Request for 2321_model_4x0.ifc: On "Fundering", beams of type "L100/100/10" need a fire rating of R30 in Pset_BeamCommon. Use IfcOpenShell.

First a look at what the model holds.

```python
import ifcopenshell
import ifcopenshell.util.element

model = ifcopenshell.open("2321_model_4x0.ifc")
print(model.schema)
storey = next(s for s in model.by_type("IfcBuildingStorey") if s.Name == "Fundering")
beams = [e for e in ifcopenshell.util.element.get_decomposition(storey) if e.is_a("IfcBeam")]
seen = {}
for e in beams:
    element_type = ifcopenshell.util.element.get_type(e)
    key = (element_type.Name if element_type != e and element_type else None, ifcopenshell.util.element.get_pset(e, "Pset_BeamCommon", "FireRating"))
    seen[key] = seen.get(key, 0) + 1
for (name, value), count in sorted(seen.items(), key=str):
    print(count, "x", name, "|", value)
```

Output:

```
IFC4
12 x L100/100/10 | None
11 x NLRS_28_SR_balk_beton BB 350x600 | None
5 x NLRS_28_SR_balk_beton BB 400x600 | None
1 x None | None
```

```python
import ifcopenshell
import ifcopenshell.api.pset
import ifcopenshell.util.element

model = ifcopenshell.open("2321_model_4x0.ifc")

storey = next(s for s in model.by_type("IfcBuildingStorey") if s.Name == "Fundering")
beams = [e for e in ifcopenshell.util.element.get_decomposition(storey) if e.is_a("IfcBeam")]

count = 0
for e in beams:
    element_type = ifcopenshell.util.element.get_type(e)
    if element_type in (None, e) or element_type.Name != "L100/100/10":
        continue
    # add_pset returns the element's existing set when there is one.
    pset = ifcopenshell.api.pset.add_pset(model, product=e, name="Pset_BeamCommon")
    ifcopenshell.api.pset.edit_pset(model, pset=pset, properties={"FireRating": "R30"})
    count += 1

print(count, "beams updated")

model.write("2321_model_4x0_edited.ifc")
```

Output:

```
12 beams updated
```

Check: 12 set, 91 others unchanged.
